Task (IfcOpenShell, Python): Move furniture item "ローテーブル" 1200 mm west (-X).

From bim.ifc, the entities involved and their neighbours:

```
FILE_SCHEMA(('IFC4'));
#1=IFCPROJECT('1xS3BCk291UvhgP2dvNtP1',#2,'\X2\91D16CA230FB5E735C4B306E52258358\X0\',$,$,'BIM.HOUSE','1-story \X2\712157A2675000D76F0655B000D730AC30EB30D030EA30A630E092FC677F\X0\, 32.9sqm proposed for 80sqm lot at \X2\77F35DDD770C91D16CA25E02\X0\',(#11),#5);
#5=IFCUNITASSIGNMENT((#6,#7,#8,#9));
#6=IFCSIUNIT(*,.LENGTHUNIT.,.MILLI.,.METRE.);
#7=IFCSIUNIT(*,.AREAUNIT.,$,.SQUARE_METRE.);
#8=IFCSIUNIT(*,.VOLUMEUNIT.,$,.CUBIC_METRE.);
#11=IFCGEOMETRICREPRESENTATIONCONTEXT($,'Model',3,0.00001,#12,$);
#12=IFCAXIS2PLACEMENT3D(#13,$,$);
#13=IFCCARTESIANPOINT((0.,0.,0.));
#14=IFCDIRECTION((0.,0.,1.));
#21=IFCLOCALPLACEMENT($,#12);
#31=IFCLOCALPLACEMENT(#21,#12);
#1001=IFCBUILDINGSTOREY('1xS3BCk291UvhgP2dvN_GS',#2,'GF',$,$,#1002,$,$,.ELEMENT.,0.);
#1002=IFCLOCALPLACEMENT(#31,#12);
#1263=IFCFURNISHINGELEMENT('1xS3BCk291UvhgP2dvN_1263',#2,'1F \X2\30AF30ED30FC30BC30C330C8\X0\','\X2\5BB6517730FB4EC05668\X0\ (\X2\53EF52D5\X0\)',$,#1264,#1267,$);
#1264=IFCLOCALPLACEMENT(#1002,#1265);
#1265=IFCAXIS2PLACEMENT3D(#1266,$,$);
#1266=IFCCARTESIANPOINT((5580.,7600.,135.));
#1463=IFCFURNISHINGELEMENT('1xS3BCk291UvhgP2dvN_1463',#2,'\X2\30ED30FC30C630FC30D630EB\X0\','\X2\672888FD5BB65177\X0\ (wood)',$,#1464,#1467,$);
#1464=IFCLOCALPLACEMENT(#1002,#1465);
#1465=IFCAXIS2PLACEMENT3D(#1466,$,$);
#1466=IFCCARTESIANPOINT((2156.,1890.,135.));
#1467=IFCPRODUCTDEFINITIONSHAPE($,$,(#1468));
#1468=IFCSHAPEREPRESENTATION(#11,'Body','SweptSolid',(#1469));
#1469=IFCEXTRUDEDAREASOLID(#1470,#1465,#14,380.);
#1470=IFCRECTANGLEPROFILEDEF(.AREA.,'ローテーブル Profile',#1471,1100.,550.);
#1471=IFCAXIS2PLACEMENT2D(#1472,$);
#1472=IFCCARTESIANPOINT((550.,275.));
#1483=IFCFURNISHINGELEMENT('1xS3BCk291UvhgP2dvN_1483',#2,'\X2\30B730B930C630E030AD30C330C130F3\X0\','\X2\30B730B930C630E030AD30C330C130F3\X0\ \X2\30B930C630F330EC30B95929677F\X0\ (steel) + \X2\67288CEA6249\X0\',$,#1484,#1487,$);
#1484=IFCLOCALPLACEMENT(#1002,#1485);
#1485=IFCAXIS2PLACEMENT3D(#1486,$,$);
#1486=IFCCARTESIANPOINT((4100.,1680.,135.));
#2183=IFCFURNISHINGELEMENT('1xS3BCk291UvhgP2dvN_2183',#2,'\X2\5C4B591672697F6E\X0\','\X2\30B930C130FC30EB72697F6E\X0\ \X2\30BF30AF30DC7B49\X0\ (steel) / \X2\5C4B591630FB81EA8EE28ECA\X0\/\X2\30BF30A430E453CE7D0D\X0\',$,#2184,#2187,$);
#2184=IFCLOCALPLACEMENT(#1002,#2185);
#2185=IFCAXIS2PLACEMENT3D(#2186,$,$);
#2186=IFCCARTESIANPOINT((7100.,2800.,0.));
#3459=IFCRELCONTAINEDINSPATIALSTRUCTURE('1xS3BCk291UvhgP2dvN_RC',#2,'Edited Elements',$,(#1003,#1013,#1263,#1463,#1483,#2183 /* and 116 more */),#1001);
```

```python
import ifcopenshell
import ifcopenshell.api.geometry
import ifcopenshell.util.placement
import ifcopenshell.util.unit

model = ifcopenshell.open("bim.ifc")
unit_scale = ifcopenshell.util.unit.calculate_unit_scale(model)

item = model.by_id(1463)
matrix = ifcopenshell.util.placement.get_local_placement(item.ObjectPlacement)
matrix[0, 3] -= 1.2 / unit_scale
ifcopenshell.api.geometry.edit_object_placement(model, product=item, matrix=matrix, is_si=False)

print(ifcopenshell.util.placement.get_local_placement(item.ObjectPlacement).round(3) + 0.0)

model.write("bim_v2.ifc")
```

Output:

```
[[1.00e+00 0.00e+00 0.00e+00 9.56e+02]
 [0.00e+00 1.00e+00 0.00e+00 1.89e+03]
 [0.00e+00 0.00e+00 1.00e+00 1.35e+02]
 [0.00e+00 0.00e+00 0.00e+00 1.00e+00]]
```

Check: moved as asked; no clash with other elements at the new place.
